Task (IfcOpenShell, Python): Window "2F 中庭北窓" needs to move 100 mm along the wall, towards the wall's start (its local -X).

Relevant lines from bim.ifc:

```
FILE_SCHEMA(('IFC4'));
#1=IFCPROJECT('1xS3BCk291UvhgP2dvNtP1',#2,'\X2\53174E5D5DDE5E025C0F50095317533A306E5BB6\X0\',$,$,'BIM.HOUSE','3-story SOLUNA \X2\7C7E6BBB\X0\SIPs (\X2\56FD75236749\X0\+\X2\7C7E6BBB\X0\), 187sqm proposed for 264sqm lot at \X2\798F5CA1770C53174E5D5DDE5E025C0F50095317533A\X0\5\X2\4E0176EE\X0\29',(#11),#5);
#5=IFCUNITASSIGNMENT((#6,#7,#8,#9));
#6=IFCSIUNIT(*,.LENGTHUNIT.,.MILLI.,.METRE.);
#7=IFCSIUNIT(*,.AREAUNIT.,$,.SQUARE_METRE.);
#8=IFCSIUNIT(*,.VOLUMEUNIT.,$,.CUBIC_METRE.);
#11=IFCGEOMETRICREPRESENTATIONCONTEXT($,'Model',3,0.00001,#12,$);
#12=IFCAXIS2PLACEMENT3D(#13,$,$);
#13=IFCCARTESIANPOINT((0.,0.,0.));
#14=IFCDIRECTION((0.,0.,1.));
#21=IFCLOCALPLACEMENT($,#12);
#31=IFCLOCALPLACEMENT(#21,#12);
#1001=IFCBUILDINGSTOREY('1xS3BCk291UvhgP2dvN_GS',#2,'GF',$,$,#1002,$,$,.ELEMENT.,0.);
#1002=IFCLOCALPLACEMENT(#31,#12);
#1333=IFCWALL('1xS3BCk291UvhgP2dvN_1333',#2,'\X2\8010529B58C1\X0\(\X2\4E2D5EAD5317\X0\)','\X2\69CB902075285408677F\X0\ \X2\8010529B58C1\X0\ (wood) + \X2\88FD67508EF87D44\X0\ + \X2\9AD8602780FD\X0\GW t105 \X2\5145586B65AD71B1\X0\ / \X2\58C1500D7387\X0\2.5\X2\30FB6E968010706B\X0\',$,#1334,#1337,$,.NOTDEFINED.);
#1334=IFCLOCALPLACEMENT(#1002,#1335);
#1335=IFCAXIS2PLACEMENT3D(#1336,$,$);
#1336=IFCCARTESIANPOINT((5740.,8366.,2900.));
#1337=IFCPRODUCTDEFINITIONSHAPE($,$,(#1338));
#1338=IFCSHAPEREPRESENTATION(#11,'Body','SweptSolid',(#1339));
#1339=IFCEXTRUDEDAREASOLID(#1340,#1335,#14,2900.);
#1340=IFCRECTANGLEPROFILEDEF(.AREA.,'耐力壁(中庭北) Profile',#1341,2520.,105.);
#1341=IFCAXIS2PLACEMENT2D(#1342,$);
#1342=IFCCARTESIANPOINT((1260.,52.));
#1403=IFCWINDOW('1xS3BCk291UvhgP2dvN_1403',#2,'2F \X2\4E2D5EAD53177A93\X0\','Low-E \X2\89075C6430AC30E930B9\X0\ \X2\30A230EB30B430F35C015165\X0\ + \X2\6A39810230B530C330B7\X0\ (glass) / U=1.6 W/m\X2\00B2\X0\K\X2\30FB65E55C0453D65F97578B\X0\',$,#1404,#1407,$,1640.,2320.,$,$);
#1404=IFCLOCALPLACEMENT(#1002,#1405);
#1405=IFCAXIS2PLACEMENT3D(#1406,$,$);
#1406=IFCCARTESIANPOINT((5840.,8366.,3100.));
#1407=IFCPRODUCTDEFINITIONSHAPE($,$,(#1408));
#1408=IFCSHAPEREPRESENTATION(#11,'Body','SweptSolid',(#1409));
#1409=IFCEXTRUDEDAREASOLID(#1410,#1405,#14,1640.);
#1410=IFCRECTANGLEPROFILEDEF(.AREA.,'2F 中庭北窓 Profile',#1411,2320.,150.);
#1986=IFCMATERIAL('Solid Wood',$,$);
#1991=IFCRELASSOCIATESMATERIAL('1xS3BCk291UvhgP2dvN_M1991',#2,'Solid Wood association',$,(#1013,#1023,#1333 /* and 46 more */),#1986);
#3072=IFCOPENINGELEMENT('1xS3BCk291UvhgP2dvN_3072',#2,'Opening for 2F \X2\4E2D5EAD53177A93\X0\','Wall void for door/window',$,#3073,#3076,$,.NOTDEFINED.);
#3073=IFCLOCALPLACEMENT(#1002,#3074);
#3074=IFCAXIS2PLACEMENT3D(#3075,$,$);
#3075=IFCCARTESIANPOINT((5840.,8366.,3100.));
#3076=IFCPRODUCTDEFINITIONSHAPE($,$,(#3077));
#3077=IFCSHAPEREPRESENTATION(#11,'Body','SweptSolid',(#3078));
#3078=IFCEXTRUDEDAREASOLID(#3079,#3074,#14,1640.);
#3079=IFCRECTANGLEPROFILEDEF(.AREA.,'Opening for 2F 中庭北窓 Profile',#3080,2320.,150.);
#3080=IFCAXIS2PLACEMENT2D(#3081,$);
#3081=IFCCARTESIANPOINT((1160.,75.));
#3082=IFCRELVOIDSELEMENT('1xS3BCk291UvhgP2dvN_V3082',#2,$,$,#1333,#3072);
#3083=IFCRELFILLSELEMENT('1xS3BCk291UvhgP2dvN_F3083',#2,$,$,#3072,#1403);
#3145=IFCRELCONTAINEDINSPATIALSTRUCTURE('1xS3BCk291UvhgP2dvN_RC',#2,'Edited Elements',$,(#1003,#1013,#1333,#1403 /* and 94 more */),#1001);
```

```python
import ifcopenshell
import ifcopenshell.api.geometry
import ifcopenshell.util.placement

model = ifcopenshell.open("bim.ifc")

window = model.by_guid("1xS3BCk291UvhgP2dvN_1403")
opening = window.FillsVoids[0].RelatingOpeningElement
wall = opening.VoidsElements[0].RelatingBuildingElement

wall_matrix = ifcopenshell.util.placement.get_local_placement(wall.ObjectPlacement)
shift = wall_matrix[:3, 0] * -100.0
before = ifcopenshell.util.placement.get_local_placement(window.ObjectPlacement)[:3, 3].copy()

# The window is not placed relative to its opening, so move both.
for product in (opening, window):
    matrix = ifcopenshell.util.placement.get_local_placement(product.ObjectPlacement)
    matrix[:3, 3] += shift
    ifcopenshell.api.geometry.edit_object_placement(model, product=product, matrix=matrix, is_si=False)

after = ifcopenshell.util.placement.get_local_placement(window.ObjectPlacement)[:3, 3]
print("window moved by", (after - before).round(3) + 0.0)

model.write("bim_rev.ifc")
```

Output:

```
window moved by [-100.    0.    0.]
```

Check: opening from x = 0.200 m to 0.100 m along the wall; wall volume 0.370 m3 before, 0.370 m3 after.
